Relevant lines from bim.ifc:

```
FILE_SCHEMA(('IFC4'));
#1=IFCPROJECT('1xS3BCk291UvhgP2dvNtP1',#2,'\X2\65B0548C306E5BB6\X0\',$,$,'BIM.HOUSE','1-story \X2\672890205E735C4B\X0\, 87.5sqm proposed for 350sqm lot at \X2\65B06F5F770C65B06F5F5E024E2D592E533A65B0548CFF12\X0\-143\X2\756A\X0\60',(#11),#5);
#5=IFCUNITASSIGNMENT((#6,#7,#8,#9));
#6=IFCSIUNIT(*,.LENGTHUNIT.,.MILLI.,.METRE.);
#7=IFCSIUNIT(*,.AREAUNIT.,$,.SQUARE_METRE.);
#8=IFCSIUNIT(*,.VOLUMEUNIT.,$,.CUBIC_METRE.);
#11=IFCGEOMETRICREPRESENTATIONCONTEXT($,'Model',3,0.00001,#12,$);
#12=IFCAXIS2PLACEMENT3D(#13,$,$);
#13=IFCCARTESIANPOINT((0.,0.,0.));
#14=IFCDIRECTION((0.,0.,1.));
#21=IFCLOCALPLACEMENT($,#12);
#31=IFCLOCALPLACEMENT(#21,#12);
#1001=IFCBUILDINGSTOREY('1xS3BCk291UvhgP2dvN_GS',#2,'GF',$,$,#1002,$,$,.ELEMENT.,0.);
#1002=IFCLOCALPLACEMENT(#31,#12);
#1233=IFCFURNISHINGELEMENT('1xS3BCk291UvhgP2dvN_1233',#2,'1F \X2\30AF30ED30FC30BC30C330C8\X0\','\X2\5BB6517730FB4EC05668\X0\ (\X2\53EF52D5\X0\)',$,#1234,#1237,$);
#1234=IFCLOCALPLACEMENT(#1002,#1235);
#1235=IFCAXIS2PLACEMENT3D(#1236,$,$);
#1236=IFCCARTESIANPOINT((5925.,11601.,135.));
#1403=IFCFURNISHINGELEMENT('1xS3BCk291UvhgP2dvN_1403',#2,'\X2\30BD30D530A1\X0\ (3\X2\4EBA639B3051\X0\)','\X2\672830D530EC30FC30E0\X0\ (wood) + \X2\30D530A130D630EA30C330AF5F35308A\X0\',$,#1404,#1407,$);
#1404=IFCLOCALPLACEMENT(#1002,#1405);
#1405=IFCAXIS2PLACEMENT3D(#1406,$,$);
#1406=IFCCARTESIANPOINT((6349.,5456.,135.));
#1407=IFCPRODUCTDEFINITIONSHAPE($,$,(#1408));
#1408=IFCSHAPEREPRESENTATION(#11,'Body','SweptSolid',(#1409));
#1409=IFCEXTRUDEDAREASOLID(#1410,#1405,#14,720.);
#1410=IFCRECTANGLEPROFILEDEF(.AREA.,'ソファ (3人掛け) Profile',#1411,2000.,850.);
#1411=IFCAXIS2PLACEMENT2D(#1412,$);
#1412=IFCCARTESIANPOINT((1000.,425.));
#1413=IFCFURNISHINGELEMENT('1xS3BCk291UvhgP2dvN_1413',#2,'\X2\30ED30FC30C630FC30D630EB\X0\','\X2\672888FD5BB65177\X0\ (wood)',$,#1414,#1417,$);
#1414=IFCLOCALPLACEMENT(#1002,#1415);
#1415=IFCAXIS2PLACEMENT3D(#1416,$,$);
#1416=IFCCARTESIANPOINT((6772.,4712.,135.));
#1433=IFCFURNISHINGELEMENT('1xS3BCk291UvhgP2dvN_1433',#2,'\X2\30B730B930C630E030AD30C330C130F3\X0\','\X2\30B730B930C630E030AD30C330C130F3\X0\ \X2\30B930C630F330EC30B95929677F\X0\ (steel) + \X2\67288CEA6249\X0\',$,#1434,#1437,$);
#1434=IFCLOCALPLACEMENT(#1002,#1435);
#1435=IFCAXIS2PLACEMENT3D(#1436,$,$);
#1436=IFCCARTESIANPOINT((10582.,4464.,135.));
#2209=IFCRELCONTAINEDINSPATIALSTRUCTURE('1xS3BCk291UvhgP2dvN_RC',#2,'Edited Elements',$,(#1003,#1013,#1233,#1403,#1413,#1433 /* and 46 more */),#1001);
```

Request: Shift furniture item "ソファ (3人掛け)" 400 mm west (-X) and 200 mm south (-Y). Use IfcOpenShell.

```python
import ifcopenshell
import ifcopenshell.api.geometry
import ifcopenshell.util.placement

model = ifcopenshell.open("bim.ifc")

item = model.by_guid("1xS3BCk291UvhgP2dvN_1403")
matrix = ifcopenshell.util.placement.get_local_placement(item.ObjectPlacement)
matrix[0, 3] -= 400.0
matrix[1, 3] -= 200.0
ifcopenshell.api.geometry.edit_object_placement(model, product=item, matrix=matrix, is_si=False)

print(ifcopenshell.util.placement.get_local_placement(item.ObjectPlacement).round(3) + 0.0)

model.write("bim-out.ifc")
```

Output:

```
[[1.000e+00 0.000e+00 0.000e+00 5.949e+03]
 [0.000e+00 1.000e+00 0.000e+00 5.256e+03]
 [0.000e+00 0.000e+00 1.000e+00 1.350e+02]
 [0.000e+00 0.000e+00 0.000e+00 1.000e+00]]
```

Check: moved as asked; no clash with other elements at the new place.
